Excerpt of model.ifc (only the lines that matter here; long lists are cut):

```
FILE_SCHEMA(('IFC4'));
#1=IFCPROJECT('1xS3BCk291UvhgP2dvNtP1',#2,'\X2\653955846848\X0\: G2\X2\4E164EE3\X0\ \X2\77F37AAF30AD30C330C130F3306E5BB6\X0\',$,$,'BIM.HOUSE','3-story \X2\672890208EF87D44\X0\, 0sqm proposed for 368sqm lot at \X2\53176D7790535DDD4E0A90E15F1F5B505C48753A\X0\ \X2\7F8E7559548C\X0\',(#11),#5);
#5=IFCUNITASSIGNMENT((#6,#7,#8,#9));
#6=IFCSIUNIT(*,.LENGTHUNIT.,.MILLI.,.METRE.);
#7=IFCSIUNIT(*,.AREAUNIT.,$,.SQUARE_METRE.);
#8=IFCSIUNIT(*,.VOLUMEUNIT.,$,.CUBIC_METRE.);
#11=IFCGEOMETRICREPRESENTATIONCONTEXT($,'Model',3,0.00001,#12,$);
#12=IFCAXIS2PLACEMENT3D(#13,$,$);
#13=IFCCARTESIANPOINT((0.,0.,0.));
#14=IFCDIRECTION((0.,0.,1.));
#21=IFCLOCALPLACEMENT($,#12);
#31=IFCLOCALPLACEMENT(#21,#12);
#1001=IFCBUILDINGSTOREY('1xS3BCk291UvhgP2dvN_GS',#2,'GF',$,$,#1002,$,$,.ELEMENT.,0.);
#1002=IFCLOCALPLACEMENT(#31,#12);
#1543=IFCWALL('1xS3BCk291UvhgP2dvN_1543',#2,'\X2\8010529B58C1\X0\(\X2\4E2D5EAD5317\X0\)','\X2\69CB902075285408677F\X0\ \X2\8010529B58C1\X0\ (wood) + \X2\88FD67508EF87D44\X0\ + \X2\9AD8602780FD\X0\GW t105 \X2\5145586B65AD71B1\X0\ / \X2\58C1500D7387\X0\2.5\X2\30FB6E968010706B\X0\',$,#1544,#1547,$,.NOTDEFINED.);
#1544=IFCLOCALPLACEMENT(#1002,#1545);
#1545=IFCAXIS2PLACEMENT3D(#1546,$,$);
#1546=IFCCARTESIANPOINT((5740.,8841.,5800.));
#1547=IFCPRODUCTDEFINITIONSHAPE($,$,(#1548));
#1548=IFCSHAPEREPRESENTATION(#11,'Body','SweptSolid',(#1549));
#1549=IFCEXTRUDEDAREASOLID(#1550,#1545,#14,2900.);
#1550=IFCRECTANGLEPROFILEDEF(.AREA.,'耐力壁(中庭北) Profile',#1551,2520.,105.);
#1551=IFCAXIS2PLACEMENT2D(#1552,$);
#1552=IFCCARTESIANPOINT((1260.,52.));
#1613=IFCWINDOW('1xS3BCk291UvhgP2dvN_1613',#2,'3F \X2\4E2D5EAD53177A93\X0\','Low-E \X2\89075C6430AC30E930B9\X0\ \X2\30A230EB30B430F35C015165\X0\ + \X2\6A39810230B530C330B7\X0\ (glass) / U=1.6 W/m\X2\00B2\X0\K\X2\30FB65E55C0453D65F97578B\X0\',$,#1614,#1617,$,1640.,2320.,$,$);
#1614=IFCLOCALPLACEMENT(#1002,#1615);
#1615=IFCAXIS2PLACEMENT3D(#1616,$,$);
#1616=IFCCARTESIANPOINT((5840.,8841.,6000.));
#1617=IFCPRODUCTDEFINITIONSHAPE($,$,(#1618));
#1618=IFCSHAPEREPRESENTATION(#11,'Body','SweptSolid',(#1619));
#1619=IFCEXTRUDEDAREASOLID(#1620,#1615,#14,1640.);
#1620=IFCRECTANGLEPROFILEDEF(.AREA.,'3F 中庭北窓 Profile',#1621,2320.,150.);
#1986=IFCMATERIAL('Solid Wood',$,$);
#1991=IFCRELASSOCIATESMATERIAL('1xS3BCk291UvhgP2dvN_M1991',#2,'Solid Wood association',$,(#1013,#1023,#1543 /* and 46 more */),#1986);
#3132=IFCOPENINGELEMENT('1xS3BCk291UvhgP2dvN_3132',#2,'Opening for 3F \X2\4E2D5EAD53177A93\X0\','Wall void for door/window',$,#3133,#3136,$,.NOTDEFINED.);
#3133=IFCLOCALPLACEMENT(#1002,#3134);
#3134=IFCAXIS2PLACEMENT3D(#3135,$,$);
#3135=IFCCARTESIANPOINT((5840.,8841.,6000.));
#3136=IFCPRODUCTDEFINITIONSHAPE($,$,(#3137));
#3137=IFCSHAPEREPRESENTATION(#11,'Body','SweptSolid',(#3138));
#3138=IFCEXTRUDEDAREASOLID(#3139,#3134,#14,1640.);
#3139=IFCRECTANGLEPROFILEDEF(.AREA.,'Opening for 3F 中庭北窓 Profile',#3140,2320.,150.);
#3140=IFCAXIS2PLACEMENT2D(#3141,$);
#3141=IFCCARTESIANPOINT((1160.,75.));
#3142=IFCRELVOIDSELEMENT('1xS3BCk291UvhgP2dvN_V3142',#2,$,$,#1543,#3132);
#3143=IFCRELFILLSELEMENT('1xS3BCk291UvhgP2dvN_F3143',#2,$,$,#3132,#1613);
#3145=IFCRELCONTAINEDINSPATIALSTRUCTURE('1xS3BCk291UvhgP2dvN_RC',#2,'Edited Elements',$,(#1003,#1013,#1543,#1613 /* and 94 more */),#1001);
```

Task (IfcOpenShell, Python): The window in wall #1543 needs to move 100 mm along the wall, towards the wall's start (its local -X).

```python
import ifcopenshell
import ifcopenshell.api.geometry
import ifcopenshell.util.placement
import ifcopenshell.util.unit

model = ifcopenshell.open("model.ifc")
unit_scale = ifcopenshell.util.unit.calculate_unit_scale(model)

window = model.by_id(1613)
opening = window.FillsVoids[0].RelatingOpeningElement
wall = opening.VoidsElements[0].RelatingBuildingElement

wall_matrix = ifcopenshell.util.placement.get_local_placement(wall.ObjectPlacement)
shift = wall_matrix[:3, 0] * -0.1 / unit_scale
before = ifcopenshell.util.placement.get_local_placement(window.ObjectPlacement)[:3, 3].copy()

# The window is not placed relative to its opening, so move both.
for product in (opening, window):
    matrix = ifcopenshell.util.placement.get_local_placement(product.ObjectPlacement)
    matrix[:3, 3] += shift
    ifcopenshell.api.geometry.edit_object_placement(model, product=product, matrix=matrix, is_si=False)

after = ifcopenshell.util.placement.get_local_placement(window.ObjectPlacement)[:3, 3]
print("window moved by", (after - before).round(3) + 0.0)

model.write("model_updated.ifc")
```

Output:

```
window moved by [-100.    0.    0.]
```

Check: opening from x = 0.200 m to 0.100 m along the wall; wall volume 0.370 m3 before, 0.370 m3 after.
